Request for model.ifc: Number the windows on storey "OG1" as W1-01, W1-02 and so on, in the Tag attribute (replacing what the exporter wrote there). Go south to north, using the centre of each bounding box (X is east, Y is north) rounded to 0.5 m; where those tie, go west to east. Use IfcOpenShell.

First a look at what the model holds.

```python
import ifcopenshell
import ifcopenshell.util.element
import ifcopenshell.util.placement

model = ifcopenshell.open("model.ifc")
print(model.schema)
storey = next(s for s in model.by_type("IfcBuildingStorey") if s.Name == "OG1")
windows = [e for e in ifcopenshell.util.element.get_decomposition(storey) if e.is_a("IfcWindow")]
for e in sorted(windows, key=lambda e: e.id()):
    origin = ifcopenshell.util.placement.get_local_placement(e.ObjectPlacement)[:3, 3]
    print(e.id(), e.Tag, e.Name, origin.round(2) + 0.0, sep=" | ")
```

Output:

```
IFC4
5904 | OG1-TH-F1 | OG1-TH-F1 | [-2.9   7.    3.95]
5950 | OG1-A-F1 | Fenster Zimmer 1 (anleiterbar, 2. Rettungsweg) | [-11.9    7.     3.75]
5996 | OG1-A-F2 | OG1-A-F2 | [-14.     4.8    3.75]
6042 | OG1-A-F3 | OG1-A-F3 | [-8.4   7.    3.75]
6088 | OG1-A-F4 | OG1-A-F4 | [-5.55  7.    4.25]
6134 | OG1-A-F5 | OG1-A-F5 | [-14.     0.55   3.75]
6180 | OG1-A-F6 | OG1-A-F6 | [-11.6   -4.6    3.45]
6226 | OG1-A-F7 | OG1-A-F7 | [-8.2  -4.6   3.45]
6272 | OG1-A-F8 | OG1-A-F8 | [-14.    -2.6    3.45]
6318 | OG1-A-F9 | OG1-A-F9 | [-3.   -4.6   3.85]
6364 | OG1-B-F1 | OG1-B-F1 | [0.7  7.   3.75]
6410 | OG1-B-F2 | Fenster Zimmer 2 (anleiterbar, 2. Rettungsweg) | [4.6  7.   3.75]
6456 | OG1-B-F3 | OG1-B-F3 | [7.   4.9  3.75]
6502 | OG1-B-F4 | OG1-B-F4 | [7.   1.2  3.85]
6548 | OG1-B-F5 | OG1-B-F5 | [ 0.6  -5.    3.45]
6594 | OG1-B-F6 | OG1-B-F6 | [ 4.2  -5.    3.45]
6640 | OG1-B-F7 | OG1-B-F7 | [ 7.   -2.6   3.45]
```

```python
import ifcopenshell
import ifcopenshell.geom
import ifcopenshell.util.element
import ifcopenshell.util.shape

model = ifcopenshell.open("model.ifc")
settings = ifcopenshell.geom.settings()
settings.set("use-world-coords", True)


def centre(element):
    shape = ifcopenshell.geom.create_shape(settings, element)
    return ifcopenshell.util.shape.get_bbox_centroid(shape.geometry)


storey = next(s for s in model.by_type("IfcBuildingStorey") if s.Name == "OG1")
windows = [e for e in ifcopenshell.util.element.get_decomposition(storey) if e.is_a("IfcWindow")]

# Insertion points can sit at a corner or the storey origin, so sort by the geometry (in metres).
centres = {e: centre(e) for e in windows}
windows.sort(key=lambda e: (round(centres[e][1] / 0.5), centres[e][0]))

for i, e in enumerate(windows, start=1):
    number = f"W1-{i:02d}"
    e.Tag = number
    print(e.id(), number)

model.write("model_edited.ifc")
```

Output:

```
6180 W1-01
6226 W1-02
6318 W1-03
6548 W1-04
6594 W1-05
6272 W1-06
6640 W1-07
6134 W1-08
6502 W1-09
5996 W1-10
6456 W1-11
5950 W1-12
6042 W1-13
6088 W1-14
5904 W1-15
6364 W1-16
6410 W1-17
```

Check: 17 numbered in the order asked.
